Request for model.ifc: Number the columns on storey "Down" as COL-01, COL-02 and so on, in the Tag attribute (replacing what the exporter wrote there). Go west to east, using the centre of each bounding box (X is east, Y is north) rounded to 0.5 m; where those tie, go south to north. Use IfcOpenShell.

First a look at what the model holds.

```python
import ifcopenshell
import ifcopenshell.util.element
import ifcopenshell.util.placement

model = ifcopenshell.open("model.ifc")
print(model.schema)
storey = next(s for s in model.by_type("IfcBuildingStorey") if s.Name == "Down")
columns = [e for e in ifcopenshell.util.element.get_decomposition(storey) if e.is_a("IfcColumn")]
for e in sorted(columns, key=lambda e: e.id()):
    origin = ifcopenshell.util.placement.get_local_placement(e.ObjectPlacement)[:3, 3]
    print(e.id(), e.Tag, e.Name, origin.round(2) + 0.0, sep=" | ")
```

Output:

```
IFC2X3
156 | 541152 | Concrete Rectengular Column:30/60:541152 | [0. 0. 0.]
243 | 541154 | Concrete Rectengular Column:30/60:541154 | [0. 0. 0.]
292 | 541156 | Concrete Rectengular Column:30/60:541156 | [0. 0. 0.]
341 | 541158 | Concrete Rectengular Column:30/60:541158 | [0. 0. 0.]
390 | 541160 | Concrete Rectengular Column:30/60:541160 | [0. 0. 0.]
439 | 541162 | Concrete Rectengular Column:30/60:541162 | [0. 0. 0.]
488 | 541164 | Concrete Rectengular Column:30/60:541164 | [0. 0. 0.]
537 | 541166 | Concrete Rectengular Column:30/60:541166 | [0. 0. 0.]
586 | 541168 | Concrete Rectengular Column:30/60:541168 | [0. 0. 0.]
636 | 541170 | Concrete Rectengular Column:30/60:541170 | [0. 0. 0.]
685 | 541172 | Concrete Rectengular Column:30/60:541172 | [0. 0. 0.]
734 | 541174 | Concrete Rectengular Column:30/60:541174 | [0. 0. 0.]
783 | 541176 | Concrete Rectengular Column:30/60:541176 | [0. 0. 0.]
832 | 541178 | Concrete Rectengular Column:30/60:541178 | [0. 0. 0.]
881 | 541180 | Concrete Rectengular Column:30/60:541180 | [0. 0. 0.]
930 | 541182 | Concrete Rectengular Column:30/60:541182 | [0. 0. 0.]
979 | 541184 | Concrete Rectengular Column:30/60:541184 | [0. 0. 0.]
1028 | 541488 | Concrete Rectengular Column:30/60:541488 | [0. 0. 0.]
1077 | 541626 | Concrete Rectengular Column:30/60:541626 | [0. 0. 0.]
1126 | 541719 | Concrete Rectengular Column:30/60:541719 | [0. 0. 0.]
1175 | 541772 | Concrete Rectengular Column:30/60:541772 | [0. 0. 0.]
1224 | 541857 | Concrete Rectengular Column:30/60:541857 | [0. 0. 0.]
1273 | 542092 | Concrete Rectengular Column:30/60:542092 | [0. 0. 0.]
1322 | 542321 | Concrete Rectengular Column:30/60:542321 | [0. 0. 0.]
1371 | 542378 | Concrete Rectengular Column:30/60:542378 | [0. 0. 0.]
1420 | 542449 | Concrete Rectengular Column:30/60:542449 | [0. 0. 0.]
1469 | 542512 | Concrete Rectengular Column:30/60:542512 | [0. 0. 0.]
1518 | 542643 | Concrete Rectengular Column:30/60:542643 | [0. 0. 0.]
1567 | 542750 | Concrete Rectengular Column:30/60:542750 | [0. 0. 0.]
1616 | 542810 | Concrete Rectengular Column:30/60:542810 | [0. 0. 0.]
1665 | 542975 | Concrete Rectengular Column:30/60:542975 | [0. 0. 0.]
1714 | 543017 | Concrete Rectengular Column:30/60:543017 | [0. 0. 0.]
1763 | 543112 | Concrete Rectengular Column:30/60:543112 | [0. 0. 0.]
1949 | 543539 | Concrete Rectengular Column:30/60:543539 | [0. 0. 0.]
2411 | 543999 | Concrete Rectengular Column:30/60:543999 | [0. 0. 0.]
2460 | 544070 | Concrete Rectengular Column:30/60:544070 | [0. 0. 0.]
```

```python
import ifcopenshell
import ifcopenshell.geom
import ifcopenshell.util.element
import ifcopenshell.util.shape

model = ifcopenshell.open("model.ifc")
settings = ifcopenshell.geom.settings()
settings.set("use-world-coords", True)


def centre(element):
    shape = ifcopenshell.geom.create_shape(settings, element)
    return ifcopenshell.util.shape.get_bbox_centroid(shape.geometry)


storey = next(s for s in model.by_type("IfcBuildingStorey") if s.Name == "Down")
columns = [e for e in ifcopenshell.util.element.get_decomposition(storey) if e.is_a("IfcColumn")]

# Insertion points can sit at a corner or the storey origin, so sort by the geometry (in metres).
centres = {e: centre(e) for e in columns}
columns.sort(key=lambda e: (round(centres[e][0] / 0.5), centres[e][1]))

for i, e in enumerate(columns, start=1):
    number = f"COL-{i:02d}"
    e.Tag = number
    print(e.id(), number)

model.write("model_v2.ifc")
```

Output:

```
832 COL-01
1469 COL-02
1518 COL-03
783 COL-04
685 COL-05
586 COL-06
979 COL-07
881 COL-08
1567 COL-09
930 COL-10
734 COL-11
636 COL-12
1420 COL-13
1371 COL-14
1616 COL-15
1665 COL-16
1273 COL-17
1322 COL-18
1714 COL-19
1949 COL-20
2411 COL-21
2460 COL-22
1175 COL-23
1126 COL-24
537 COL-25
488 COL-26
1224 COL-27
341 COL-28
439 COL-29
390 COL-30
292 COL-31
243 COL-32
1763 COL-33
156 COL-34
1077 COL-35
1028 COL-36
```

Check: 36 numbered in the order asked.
